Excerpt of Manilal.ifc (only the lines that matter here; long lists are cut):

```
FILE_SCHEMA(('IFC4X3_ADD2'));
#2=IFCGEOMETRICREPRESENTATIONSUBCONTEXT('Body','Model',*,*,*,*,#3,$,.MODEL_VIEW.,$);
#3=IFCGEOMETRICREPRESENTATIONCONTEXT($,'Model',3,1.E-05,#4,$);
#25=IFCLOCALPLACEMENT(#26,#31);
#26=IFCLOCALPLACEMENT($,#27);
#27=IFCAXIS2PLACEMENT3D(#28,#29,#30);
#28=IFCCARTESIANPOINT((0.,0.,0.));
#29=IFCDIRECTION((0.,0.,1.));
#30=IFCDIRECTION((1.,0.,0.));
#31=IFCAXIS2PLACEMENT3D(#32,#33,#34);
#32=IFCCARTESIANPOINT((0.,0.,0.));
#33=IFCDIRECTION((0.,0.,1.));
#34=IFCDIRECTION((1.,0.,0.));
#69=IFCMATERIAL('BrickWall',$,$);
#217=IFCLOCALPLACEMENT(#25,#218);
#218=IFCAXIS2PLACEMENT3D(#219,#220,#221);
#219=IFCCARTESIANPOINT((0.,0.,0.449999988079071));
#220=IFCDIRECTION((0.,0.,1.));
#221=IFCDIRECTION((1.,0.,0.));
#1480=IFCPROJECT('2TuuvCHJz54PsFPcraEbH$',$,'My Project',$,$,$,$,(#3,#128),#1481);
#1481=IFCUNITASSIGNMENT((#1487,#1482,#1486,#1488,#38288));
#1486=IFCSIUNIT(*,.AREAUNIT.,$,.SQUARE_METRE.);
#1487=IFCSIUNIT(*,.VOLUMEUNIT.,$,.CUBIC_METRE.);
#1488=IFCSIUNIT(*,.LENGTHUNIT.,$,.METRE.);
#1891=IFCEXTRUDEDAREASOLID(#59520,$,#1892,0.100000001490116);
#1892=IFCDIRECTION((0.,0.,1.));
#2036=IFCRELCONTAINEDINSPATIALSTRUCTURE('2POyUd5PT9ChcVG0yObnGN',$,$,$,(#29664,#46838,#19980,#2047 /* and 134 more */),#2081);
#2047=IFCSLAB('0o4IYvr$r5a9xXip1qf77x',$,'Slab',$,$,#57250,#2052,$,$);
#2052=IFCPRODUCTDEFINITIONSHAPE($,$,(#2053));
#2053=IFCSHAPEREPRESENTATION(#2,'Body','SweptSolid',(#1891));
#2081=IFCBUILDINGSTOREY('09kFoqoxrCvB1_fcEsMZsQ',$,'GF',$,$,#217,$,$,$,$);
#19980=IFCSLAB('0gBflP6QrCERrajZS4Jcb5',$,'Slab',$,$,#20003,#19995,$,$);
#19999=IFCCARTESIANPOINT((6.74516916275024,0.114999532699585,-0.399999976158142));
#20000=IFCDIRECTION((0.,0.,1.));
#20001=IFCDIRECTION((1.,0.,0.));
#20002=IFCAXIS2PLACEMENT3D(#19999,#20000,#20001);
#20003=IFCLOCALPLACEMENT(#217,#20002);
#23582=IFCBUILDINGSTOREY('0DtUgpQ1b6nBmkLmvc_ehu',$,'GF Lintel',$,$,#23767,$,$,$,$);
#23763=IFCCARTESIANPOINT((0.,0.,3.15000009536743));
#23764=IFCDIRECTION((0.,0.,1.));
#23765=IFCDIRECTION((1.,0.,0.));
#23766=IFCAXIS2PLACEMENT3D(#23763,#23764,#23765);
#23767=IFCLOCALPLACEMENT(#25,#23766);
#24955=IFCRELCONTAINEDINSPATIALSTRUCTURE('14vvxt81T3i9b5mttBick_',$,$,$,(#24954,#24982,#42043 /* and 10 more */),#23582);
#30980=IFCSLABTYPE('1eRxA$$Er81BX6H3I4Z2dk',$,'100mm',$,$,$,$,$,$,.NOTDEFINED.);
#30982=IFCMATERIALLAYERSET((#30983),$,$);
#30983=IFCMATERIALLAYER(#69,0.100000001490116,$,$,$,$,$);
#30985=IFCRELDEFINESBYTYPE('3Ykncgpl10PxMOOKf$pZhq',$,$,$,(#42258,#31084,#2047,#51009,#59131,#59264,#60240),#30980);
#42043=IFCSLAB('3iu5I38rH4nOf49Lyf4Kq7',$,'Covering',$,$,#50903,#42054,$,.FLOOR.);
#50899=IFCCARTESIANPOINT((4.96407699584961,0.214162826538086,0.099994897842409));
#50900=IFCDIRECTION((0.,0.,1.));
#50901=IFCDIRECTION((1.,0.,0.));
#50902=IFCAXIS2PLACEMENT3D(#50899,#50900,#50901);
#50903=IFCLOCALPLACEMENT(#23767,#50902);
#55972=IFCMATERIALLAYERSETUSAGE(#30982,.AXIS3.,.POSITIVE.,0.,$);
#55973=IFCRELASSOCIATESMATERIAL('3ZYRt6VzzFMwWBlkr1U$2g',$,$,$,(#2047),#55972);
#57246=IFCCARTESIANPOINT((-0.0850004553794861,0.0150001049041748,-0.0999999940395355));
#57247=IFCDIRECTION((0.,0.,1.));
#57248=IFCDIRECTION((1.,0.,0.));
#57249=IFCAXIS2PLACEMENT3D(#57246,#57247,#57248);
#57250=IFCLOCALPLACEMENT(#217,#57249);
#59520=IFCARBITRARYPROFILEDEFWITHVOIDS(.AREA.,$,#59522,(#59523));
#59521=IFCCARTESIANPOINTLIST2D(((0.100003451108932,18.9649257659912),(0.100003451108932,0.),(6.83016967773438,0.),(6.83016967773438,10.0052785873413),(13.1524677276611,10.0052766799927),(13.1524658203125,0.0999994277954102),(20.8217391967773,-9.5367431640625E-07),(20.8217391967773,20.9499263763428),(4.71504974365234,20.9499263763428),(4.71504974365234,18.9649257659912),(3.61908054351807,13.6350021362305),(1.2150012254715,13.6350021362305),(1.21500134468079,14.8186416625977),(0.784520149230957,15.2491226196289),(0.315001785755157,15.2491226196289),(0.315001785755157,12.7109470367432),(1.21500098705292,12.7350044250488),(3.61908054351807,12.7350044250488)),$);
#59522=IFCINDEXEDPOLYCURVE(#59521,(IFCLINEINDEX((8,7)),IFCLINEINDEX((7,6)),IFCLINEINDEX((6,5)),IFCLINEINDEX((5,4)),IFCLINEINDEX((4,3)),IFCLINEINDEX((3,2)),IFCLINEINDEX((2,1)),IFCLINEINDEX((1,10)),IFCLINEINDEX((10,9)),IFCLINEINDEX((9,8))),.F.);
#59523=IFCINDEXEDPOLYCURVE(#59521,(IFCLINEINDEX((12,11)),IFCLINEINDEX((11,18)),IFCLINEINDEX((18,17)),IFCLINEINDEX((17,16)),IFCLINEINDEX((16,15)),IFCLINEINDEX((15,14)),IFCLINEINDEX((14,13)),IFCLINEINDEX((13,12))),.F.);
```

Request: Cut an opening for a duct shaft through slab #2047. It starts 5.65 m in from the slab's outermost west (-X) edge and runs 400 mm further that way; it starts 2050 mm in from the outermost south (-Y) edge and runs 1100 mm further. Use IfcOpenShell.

```python
import numpy as np
import ifcopenshell
import ifcopenshell.api.feature
import ifcopenshell.api.geometry
import ifcopenshell.api.root
import ifcopenshell.geom
import ifcopenshell.util.placement
import ifcopenshell.util.representation
import ifcopenshell.util.shape
import ifcopenshell.util.unit

model = ifcopenshell.open("Manilal.ifc")
unit_scale = ifcopenshell.util.unit.calculate_unit_scale(model)
settings = ifcopenshell.geom.settings()


def volume(element):
    """Net volume in cubic metres, openings subtracted."""
    shape = ifcopenshell.geom.create_shape(settings, element)
    return ifcopenshell.util.shape.get_volume(shape.geometry)


slab = model.by_guid("0o4IYvr$r5a9xXip1qf77x")
before = volume(slab)

# Extent in the slab's own axes, in metres. The edges named are its -X and -Y sides.
slab_shape = ifcopenshell.geom.create_shape(settings, slab)
vertices = ifcopenshell.util.shape.get_vertices(slab_shape.geometry)
x_min, y_min, bottom = vertices.min(axis=0)
top = vertices[:, 2].max()

opening = ifcopenshell.api.root.create_entity(model, ifc_class="IfcOpeningElement", name="Duct shaft opening", predefined_type="OPENING")
context = ifcopenshell.util.representation.get_context(model, "Model", "Body", "MODEL_VIEW")
width, depth = 0.4, 1.1
outline = [(0.0, 0.0), (width, 0.0), (width, depth), (0.0, depth), (0.0, 0.0)]
# Overshoot both faces by 50 mm so the cut is clean.
shape = ifcopenshell.api.geometry.add_slab_representation(
    model, context=context, depth=top - bottom + 0.1, polyline=outline
)
ifcopenshell.api.geometry.assign_representation(model, product=opening, representation=shape)

matrix = ifcopenshell.util.placement.get_local_placement(slab.ObjectPlacement)
matrix[:, 3] = matrix @ np.append(np.array([x_min + 5.65, y_min + 2.05, bottom - 0.05]) / unit_scale, 1.0)
ifcopenshell.api.geometry.edit_object_placement(model, product=opening, matrix=matrix, is_si=False)
ifcopenshell.api.feature.add_feature(model, feature=opening, element=slab)

after = volume(slab)

print(f"slab volume {before:.3f} -> {after:.3f} m3")

model.write("Manilal_updated.ifc")
```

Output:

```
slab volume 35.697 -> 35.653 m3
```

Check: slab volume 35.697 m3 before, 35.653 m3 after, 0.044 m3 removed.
